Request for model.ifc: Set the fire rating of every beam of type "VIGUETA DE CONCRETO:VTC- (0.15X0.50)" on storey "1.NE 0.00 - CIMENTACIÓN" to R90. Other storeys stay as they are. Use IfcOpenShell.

First a look at what the model holds.

```python
import ifcopenshell
import ifcopenshell.util.element

model = ifcopenshell.open("model.ifc")
print(model.schema)
storey = next(s for s in model.by_type("IfcBuildingStorey") if s.Name == "1.NE 0.00 - CIMENTACIÓN")
beams = [e for e in ifcopenshell.util.element.get_decomposition(storey) if e.is_a("IfcBeam")]
seen = {}
for e in beams:
    element_type = ifcopenshell.util.element.get_type(e)
    key = (element_type.Name if element_type != e and element_type else None, ifcopenshell.util.element.get_pset(e, "Pset_BeamCommon", "FireRating"))
    seen[key] = seen.get(key, 0) + 1
for (name, value), count in sorted(seen.items(), key=str):
    print(count, "x", name, "|", value)
```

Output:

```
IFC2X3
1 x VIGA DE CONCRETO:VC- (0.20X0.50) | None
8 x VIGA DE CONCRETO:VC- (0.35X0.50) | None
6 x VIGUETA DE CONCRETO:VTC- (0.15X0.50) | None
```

```python
import ifcopenshell
import ifcopenshell.api.pset
import ifcopenshell.util.element

model = ifcopenshell.open("model.ifc")

storey = next(s for s in model.by_type("IfcBuildingStorey") if s.Name == "1.NE 0.00 - CIMENTACIÓN")
beams = [e for e in ifcopenshell.util.element.get_decomposition(storey) if e.is_a("IfcBeam")]

count = 0
for e in beams:
    element_type = ifcopenshell.util.element.get_type(e)
    if element_type in (None, e) or element_type.Name != "VIGUETA DE CONCRETO:VTC- (0.15X0.50)":
        continue
    # add_pset returns the element's existing set when there is one.
    pset = ifcopenshell.api.pset.add_pset(model, product=e, name="Pset_BeamCommon")
    ifcopenshell.api.pset.edit_pset(model, pset=pset, properties={"FireRating": "R90"})
    count += 1

print(count, "beams updated")

model.write("model-out.ifc")
```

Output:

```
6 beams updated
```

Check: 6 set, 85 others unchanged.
